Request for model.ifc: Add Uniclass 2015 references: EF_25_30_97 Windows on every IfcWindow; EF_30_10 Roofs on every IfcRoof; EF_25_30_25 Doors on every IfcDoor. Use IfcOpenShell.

First a look at what the model holds.

```python
import ifcopenshell

model = ifcopenshell.open("model.ifc")
print(model.schema)
print("classifications:", [c.Name for c in model.by_type("IfcClassification")])
for ifc_class in ("IfcDoor", "IfcRoof", "IfcStair", "IfcWall", "IfcWindow"):
    print(ifc_class, len(model.by_type(ifc_class)))
```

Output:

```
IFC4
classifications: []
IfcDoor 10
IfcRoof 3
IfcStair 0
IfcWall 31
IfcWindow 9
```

```python
import ifcopenshell
import ifcopenshell.api.classification

model = ifcopenshell.open("model.ifc")

system = ifcopenshell.api.classification.add_classification(model, classification="Uniclass 2015")

codes = {
    "IfcWindow": ("EF_25_30_97", "Windows"),
    "IfcRoof": ("EF_30_10", "Roofs"),
    "IfcDoor": ("EF_25_30_25", "Doors"),
}
for ifc_class, (code, name) in codes.items():
    products = model.by_type(ifc_class)
    ifcopenshell.api.classification.add_reference(
        model, products=products, classification=system, identification=code, name=name
    )
    print(code, len(products))

model.write("model_updated.ifc")
```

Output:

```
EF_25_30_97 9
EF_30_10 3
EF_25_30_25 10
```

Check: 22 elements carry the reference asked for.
